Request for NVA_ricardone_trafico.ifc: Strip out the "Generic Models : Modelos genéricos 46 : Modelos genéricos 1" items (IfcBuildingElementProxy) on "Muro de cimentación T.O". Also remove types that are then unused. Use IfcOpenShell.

First a look at what the model holds.

```python
import ifcopenshell
import ifcopenshell.util.element

model = ifcopenshell.open("NVA_ricardone_trafico.ifc")
print(model.schema)
storey = next(s for s in model.by_type("IfcBuildingStorey") if s.Name == "Muro de cimentación T.O")
proxies = [e for e in ifcopenshell.util.element.get_decomposition(storey) if e.is_a("IfcBuildingElementProxy")]
seen = {}
for e in proxies:
    element_type = ifcopenshell.util.element.get_type(e)
    name = element_type.Name if element_type not in (None, e) else None
    seen[name] = seen.get(name, 0) + 1
for name, count in sorted(seen.items(), key=str):
    print(count, "x", name)
```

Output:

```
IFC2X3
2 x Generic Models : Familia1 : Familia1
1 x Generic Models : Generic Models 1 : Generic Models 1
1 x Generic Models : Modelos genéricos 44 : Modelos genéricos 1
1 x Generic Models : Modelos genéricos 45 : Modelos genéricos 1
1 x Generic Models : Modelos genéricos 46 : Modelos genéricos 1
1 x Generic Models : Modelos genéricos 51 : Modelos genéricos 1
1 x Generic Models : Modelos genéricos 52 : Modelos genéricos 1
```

```python
import ifcopenshell
import ifcopenshell.api.root
import ifcopenshell.util.element

model = ifcopenshell.open("NVA_ricardone_trafico.ifc")

storey = next(s for s in model.by_type("IfcBuildingStorey") if s.Name == "Muro de cimentación T.O")
proxies = [e for e in ifcopenshell.util.element.get_decomposition(storey) if e.is_a("IfcBuildingElementProxy")]
targets = [e for e in proxies if (t := ifcopenshell.util.element.get_type(e)) not in (None, e) and t.Name == "Generic Models : Modelos genéricos 46 : Modelos genéricos 1"]
types = {ifcopenshell.util.element.get_type(e) for e in targets} - {None, *targets}

for e in targets:
    ifcopenshell.api.root.remove_product(model, product=e)
print(len(targets), "removed")

unused = [t for t in types if not ifcopenshell.util.element.get_types(t)]
for t in unused:
    ifcopenshell.api.root.remove_product(model, product=t)
print(len(unused), "unused types removed")

model.write("NVA_ricardone_trafico-out.ifc")
```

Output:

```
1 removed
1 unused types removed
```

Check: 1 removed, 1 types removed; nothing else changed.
